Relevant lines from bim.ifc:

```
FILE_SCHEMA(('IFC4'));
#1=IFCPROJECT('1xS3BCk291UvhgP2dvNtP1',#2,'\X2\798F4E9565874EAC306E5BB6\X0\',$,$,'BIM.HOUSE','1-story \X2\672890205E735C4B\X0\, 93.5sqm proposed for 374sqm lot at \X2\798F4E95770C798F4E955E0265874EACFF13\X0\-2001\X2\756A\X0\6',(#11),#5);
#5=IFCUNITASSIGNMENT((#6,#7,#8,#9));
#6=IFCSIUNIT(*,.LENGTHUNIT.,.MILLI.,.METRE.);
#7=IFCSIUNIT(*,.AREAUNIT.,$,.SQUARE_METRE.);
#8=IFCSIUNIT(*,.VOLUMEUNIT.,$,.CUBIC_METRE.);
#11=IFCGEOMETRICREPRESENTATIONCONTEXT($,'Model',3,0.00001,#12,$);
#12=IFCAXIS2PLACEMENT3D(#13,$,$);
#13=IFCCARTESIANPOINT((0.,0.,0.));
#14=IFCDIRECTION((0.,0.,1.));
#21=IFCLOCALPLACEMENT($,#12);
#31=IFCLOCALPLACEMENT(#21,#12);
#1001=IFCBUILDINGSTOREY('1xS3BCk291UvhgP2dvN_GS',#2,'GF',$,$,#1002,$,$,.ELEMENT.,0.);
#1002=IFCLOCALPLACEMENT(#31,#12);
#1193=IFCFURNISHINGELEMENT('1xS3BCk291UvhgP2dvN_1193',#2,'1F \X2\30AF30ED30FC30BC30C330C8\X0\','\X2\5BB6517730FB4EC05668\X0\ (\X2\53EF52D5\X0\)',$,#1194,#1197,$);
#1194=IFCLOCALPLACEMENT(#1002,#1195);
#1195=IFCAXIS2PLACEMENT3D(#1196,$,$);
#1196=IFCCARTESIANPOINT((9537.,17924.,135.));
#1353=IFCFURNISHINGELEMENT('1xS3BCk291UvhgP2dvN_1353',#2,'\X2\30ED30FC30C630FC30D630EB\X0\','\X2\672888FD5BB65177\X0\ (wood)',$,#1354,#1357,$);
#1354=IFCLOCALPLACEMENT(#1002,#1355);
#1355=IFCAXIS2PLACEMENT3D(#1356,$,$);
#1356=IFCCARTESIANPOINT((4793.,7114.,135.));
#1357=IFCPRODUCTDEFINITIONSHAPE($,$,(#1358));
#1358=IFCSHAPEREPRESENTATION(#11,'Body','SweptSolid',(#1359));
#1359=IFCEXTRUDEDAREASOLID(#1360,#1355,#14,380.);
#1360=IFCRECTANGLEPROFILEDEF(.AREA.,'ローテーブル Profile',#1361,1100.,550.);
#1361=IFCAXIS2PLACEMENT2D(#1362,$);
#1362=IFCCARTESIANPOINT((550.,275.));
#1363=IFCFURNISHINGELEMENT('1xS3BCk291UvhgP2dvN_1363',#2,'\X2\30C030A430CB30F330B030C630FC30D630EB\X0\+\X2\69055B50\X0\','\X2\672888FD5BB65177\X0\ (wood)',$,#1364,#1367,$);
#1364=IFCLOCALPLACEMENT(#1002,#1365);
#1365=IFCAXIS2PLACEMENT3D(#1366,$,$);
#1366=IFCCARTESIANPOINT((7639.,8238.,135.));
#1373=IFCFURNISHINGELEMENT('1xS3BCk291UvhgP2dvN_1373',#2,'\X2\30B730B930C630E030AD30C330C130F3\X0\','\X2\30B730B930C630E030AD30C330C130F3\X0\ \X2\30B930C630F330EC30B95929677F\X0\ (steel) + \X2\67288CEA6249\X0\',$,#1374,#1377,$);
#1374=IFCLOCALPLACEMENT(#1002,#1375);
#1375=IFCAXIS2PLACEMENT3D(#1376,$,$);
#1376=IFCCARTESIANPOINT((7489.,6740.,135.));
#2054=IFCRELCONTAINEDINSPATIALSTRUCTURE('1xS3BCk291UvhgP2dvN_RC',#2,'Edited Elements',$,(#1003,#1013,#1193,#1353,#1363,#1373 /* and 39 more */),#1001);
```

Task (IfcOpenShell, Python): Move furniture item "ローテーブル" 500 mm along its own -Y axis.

```python
import ifcopenshell
import ifcopenshell.api.geometry
import ifcopenshell.util.placement

model = ifcopenshell.open("bim.ifc")

item = model.by_guid("1xS3BCk291UvhgP2dvN_1353")
matrix = ifcopenshell.util.placement.get_local_placement(item.ObjectPlacement)
matrix[:3, 3] -= matrix[:3, 1] * 500.0
ifcopenshell.api.geometry.edit_object_placement(model, product=item, matrix=matrix, is_si=False)

print(ifcopenshell.util.placement.get_local_placement(item.ObjectPlacement).round(3) + 0.0)

model.write("bim_updated.ifc")
```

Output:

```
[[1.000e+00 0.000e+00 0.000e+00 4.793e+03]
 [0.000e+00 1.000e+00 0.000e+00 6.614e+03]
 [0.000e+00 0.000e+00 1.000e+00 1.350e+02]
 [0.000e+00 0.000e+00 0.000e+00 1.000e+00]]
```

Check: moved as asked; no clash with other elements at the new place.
